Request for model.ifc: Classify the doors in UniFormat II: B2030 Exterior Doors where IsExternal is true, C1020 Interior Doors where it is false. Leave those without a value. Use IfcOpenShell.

First a look at what the model holds.

```python
import ifcopenshell
import ifcopenshell.util.element

model = ifcopenshell.open("model.ifc")
print(model.schema)
print("classifications:", [c.Name for c in model.by_type("IfcClassification")])
values = [ifcopenshell.util.element.get_pset(e, "Pset_DoorCommon", "IsExternal") for e in model.by_type("IfcDoor")]
for value in (True, False, None):
    print("IsExternal", value, values.count(value))
```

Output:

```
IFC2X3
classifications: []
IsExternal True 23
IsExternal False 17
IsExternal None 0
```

```python
import ifcopenshell
import ifcopenshell.api.classification
import ifcopenshell.util.element

model = ifcopenshell.open("model.ifc")

# IFC2X3 requires Source and Edition and has no link from the project to the system.
system = model.create_entity("IfcClassification", Source="ASTM", Edition="E1557", Name="UniFormat II")

doors = model.by_type("IfcDoor")
external = {e: ifcopenshell.util.element.get_pset(e, "Pset_DoorCommon", "IsExternal") for e in doors}
for flag, code, name in ((True, "B2030", "Exterior Doors"), (False, "C1020", "Interior Doors")):
    products = [e for e in doors if external[e] is flag]
    ifcopenshell.api.classification.add_reference(
        model, products=products, classification=system, identification=code, name=name
    )
    print(code, len(products))

model.write("model_v2.ifc")
```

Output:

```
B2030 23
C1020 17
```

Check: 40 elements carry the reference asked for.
